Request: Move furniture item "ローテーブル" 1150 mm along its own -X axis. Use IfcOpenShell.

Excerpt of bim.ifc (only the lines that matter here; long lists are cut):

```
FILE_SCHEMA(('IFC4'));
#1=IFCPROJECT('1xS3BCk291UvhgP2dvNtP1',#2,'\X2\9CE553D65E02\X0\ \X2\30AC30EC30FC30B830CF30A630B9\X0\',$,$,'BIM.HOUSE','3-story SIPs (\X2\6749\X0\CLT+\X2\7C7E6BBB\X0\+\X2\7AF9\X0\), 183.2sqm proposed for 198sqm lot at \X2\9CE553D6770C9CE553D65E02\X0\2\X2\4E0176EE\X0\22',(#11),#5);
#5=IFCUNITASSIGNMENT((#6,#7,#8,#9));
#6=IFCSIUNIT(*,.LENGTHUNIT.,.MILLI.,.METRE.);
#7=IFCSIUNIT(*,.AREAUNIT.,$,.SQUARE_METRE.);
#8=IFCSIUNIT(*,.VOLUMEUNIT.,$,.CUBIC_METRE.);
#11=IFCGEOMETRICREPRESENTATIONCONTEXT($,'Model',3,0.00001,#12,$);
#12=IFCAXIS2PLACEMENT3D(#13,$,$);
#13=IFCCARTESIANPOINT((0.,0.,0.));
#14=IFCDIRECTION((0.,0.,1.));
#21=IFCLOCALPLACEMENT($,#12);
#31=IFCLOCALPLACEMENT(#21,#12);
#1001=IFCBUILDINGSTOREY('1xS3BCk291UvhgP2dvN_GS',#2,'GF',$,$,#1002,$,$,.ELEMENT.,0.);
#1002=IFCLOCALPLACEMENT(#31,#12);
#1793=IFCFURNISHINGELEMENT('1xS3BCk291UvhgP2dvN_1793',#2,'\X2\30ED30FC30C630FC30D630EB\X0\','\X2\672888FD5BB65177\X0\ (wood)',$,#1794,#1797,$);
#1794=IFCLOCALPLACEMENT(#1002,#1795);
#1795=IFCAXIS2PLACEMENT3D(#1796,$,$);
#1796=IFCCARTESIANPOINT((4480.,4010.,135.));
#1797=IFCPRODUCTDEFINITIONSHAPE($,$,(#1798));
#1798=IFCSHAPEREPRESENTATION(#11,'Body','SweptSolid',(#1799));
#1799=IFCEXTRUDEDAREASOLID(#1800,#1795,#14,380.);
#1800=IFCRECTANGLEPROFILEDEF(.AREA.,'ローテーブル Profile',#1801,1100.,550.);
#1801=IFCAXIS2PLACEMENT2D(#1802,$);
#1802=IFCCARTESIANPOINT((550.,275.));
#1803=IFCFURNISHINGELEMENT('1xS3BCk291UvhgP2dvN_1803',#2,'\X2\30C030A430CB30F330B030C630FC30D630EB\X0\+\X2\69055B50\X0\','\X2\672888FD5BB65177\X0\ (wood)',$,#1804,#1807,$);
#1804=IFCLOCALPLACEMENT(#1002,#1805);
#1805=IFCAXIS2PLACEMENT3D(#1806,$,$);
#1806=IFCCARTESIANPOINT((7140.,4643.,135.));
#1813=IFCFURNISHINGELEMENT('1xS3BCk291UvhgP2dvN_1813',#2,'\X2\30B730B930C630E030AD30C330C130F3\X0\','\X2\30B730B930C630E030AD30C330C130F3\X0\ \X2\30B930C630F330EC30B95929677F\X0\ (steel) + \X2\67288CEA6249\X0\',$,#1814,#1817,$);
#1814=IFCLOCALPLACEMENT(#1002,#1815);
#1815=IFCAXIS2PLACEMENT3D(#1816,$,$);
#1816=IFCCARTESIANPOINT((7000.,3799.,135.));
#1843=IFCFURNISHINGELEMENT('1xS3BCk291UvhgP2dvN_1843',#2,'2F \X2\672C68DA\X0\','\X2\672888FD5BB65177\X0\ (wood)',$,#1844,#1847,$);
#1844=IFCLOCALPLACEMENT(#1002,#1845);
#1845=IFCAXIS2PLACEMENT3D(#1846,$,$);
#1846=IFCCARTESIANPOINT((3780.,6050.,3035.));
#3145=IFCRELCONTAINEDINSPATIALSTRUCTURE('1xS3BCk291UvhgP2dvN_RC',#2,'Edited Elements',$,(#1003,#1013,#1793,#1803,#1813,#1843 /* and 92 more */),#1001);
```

```python
import ifcopenshell
import ifcopenshell.api.geometry
import ifcopenshell.util.placement

model = ifcopenshell.open("bim.ifc")

item = model.by_guid("1xS3BCk291UvhgP2dvN_1793")
matrix = ifcopenshell.util.placement.get_local_placement(item.ObjectPlacement)
matrix[:3, 3] -= matrix[:3, 0] * 1150.0
ifcopenshell.api.geometry.edit_object_placement(model, product=item, matrix=matrix, is_si=False)

print(ifcopenshell.util.placement.get_local_placement(item.ObjectPlacement).round(3) + 0.0)

model.write("bim_updated.ifc")
```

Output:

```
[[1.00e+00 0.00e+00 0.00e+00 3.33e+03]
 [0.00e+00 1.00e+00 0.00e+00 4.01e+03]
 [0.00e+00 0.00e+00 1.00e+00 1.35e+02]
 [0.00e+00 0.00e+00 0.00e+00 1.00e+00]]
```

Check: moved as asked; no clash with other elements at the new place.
